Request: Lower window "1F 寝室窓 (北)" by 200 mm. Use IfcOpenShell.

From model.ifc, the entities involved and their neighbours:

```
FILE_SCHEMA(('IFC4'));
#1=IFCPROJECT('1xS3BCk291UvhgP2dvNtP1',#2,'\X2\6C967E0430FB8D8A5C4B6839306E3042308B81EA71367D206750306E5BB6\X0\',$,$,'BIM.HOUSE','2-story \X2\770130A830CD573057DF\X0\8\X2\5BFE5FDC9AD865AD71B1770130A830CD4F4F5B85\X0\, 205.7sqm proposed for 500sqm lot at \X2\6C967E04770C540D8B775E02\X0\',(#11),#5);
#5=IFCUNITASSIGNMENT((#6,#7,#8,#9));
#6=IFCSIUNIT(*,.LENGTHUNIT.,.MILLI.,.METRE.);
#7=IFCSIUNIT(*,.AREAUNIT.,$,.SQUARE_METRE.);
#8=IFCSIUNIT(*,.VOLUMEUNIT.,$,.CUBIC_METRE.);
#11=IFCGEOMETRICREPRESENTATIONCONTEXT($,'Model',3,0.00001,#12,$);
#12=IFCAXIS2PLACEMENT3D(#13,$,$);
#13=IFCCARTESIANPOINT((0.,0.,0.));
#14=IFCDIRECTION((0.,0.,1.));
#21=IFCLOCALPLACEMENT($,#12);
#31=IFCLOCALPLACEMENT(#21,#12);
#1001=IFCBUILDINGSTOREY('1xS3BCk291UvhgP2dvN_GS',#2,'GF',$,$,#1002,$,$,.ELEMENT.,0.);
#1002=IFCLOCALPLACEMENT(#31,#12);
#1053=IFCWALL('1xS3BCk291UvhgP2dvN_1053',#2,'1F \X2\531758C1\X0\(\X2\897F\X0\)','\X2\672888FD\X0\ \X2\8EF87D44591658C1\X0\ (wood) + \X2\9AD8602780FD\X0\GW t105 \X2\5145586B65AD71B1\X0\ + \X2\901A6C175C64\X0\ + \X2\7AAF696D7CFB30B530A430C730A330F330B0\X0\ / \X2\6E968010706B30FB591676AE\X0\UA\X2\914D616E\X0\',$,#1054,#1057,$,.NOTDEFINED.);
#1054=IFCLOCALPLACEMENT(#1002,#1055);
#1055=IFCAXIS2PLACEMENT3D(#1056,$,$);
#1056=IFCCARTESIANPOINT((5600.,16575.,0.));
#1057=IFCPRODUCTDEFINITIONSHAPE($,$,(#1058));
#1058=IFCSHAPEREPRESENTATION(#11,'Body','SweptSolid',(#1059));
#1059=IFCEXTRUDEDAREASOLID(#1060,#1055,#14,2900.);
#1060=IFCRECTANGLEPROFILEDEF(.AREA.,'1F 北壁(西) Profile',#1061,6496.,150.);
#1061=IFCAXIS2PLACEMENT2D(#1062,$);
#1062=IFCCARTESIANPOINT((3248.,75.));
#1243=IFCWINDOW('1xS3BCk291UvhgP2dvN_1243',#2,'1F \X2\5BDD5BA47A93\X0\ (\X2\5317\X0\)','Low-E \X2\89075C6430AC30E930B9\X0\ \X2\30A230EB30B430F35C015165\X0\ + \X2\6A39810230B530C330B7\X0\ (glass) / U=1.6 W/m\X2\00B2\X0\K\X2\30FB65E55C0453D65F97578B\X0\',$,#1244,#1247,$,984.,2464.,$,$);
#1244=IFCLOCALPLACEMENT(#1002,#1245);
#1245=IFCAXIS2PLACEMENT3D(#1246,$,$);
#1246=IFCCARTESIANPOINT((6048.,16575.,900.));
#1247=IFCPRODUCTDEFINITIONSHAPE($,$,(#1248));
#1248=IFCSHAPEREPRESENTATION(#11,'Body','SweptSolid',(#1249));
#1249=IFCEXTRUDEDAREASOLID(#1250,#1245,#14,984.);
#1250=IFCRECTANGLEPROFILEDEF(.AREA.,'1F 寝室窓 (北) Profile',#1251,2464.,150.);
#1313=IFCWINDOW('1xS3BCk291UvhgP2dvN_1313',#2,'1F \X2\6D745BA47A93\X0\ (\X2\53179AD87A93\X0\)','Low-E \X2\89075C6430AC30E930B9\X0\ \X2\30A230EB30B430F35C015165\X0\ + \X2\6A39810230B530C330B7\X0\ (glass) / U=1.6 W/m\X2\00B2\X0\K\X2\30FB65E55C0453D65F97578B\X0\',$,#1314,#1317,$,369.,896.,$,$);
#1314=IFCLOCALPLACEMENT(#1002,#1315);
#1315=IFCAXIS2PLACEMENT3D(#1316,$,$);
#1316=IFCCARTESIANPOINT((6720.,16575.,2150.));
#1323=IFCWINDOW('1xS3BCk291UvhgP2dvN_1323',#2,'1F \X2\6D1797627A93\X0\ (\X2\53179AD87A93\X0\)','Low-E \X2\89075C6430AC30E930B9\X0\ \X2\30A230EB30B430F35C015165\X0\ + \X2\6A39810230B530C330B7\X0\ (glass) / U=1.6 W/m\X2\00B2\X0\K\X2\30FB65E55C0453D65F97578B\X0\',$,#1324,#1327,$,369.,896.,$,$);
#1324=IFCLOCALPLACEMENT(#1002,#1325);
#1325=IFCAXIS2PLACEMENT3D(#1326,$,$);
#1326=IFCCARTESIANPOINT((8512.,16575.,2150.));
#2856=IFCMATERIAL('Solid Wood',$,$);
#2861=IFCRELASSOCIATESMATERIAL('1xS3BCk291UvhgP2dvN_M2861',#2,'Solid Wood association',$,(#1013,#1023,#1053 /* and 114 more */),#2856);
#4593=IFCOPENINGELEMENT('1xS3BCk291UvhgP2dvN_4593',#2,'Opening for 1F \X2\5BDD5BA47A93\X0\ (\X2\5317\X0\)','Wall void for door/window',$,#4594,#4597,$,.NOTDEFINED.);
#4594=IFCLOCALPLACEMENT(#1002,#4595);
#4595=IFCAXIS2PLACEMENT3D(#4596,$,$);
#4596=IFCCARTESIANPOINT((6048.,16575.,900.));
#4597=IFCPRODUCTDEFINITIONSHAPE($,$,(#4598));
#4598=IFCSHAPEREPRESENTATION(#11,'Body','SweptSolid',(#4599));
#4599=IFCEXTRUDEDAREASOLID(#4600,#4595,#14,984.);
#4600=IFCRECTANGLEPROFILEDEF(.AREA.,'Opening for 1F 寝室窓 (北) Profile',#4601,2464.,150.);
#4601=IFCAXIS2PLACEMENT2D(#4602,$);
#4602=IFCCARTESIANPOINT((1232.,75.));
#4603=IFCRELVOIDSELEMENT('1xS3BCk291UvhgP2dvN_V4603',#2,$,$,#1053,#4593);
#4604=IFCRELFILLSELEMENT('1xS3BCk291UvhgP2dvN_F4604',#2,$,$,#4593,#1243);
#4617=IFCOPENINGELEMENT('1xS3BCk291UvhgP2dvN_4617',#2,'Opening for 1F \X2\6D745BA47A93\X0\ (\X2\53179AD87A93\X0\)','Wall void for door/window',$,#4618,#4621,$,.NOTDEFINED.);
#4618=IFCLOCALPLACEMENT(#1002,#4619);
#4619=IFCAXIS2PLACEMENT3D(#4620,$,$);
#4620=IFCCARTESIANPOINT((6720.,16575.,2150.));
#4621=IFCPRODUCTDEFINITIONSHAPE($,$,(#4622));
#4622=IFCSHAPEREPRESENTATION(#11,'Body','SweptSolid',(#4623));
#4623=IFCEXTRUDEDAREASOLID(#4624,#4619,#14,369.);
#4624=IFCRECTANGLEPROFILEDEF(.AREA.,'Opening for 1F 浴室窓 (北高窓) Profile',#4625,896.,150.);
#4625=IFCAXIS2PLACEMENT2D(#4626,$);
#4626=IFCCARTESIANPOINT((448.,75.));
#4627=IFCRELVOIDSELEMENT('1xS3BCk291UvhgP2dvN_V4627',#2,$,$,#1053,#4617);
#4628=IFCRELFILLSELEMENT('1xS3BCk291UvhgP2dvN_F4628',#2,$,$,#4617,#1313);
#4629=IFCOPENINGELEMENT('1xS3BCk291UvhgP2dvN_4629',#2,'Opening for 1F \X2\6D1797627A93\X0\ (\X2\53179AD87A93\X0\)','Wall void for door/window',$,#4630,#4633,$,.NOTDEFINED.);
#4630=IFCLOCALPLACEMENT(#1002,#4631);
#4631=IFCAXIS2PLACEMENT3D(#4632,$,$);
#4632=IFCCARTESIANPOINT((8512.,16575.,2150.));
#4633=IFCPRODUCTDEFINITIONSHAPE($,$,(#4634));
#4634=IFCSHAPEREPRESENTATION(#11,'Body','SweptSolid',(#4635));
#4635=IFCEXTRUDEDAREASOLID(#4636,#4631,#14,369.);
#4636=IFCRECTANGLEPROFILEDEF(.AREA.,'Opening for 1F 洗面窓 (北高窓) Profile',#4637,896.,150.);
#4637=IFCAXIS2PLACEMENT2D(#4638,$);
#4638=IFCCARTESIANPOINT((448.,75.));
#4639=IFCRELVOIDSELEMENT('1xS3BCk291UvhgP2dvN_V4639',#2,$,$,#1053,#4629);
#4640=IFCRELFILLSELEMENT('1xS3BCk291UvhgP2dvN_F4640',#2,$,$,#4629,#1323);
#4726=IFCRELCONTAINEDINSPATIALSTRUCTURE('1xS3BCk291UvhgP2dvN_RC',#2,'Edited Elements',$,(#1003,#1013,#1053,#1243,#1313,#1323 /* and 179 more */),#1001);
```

```python
import numpy as np
import ifcopenshell
import ifcopenshell.api.geometry
import ifcopenshell.util.placement
import ifcopenshell.util.unit

model = ifcopenshell.open("model.ifc")
unit_scale = ifcopenshell.util.unit.calculate_unit_scale(model)

window = model.by_guid("1xS3BCk291UvhgP2dvN_1243")
opening = window.FillsVoids[0].RelatingOpeningElement
dz = -0.2 / unit_scale

shift = np.array([0.0, 0.0, dz])
# The window is not placed relative to its opening, so move both.
for product in (opening, window):
    matrix = ifcopenshell.util.placement.get_local_placement(product.ObjectPlacement)
    matrix[:3, 3] += shift
    ifcopenshell.api.geometry.edit_object_placement(model, product=product, matrix=matrix, is_si=False)

print(f"moved by {dz * unit_scale:+.3f} m")

model.write("model_edited.ifc")
```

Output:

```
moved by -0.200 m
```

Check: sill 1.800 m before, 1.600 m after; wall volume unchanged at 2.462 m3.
